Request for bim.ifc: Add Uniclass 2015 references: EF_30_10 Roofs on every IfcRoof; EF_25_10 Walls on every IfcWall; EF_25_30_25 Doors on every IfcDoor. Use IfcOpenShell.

First a look at what the model holds.

```python
import ifcopenshell

model = ifcopenshell.open("bim.ifc")
print(model.schema)
print("classifications:", [c.Name for c in model.by_type("IfcClassification")])
for ifc_class in ("IfcDoor", "IfcRoof", "IfcStair", "IfcWall", "IfcWindow"):
    print(ifc_class, len(model.by_type(ifc_class)))
```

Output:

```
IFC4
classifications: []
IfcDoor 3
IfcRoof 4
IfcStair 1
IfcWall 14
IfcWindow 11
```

```python
import ifcopenshell
import ifcopenshell.api.classification

model = ifcopenshell.open("bim.ifc")

system = ifcopenshell.api.classification.add_classification(model, classification="Uniclass 2015")

codes = {
    "IfcRoof": ("EF_30_10", "Roofs"),
    "IfcWall": ("EF_25_10", "Walls"),
    "IfcDoor": ("EF_25_30_25", "Doors"),
}
for ifc_class, (code, name) in codes.items():
    products = model.by_type(ifc_class)
    ifcopenshell.api.classification.add_reference(
        model, products=products, classification=system, identification=code, name=name
    )
    print(code, len(products))

model.write("bim_v2.ifc")
```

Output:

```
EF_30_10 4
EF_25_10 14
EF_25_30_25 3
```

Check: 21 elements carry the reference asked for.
